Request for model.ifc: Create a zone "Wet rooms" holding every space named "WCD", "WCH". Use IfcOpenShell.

First a look at what the model holds.

```python
import ifcopenshell

model = ifcopenshell.open("model.ifc")
print(model.schema)
seen = {}
for space in model.by_type("IfcSpace"):
    seen[space.LongName] = seen.get(space.LongName, 0) + 1
for name, count in sorted(seen.items(), key=str):
    print(count, "x", name)
print("zones:", [z.Name for z in model.by_type("IfcZone")][:20])
```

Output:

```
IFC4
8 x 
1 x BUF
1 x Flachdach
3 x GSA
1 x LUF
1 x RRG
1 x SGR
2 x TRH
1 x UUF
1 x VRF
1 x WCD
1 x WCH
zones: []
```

```python
import ifcopenshell
import ifcopenshell.api.group
import ifcopenshell.api.root

model = ifcopenshell.open("model.ifc")

names = {"WCD", "WCH"}
spaces = [s for s in model.by_type("IfcSpace") if s.LongName in names]

zone = ifcopenshell.api.root.create_entity(model, ifc_class="IfcZone", name="Wet rooms")
ifcopenshell.api.group.assign_group(model, products=spaces, group=zone)
print(len(spaces), "spaces in", zone.Name)

model.write("model_rev.ifc")
```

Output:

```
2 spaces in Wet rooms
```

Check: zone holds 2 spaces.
